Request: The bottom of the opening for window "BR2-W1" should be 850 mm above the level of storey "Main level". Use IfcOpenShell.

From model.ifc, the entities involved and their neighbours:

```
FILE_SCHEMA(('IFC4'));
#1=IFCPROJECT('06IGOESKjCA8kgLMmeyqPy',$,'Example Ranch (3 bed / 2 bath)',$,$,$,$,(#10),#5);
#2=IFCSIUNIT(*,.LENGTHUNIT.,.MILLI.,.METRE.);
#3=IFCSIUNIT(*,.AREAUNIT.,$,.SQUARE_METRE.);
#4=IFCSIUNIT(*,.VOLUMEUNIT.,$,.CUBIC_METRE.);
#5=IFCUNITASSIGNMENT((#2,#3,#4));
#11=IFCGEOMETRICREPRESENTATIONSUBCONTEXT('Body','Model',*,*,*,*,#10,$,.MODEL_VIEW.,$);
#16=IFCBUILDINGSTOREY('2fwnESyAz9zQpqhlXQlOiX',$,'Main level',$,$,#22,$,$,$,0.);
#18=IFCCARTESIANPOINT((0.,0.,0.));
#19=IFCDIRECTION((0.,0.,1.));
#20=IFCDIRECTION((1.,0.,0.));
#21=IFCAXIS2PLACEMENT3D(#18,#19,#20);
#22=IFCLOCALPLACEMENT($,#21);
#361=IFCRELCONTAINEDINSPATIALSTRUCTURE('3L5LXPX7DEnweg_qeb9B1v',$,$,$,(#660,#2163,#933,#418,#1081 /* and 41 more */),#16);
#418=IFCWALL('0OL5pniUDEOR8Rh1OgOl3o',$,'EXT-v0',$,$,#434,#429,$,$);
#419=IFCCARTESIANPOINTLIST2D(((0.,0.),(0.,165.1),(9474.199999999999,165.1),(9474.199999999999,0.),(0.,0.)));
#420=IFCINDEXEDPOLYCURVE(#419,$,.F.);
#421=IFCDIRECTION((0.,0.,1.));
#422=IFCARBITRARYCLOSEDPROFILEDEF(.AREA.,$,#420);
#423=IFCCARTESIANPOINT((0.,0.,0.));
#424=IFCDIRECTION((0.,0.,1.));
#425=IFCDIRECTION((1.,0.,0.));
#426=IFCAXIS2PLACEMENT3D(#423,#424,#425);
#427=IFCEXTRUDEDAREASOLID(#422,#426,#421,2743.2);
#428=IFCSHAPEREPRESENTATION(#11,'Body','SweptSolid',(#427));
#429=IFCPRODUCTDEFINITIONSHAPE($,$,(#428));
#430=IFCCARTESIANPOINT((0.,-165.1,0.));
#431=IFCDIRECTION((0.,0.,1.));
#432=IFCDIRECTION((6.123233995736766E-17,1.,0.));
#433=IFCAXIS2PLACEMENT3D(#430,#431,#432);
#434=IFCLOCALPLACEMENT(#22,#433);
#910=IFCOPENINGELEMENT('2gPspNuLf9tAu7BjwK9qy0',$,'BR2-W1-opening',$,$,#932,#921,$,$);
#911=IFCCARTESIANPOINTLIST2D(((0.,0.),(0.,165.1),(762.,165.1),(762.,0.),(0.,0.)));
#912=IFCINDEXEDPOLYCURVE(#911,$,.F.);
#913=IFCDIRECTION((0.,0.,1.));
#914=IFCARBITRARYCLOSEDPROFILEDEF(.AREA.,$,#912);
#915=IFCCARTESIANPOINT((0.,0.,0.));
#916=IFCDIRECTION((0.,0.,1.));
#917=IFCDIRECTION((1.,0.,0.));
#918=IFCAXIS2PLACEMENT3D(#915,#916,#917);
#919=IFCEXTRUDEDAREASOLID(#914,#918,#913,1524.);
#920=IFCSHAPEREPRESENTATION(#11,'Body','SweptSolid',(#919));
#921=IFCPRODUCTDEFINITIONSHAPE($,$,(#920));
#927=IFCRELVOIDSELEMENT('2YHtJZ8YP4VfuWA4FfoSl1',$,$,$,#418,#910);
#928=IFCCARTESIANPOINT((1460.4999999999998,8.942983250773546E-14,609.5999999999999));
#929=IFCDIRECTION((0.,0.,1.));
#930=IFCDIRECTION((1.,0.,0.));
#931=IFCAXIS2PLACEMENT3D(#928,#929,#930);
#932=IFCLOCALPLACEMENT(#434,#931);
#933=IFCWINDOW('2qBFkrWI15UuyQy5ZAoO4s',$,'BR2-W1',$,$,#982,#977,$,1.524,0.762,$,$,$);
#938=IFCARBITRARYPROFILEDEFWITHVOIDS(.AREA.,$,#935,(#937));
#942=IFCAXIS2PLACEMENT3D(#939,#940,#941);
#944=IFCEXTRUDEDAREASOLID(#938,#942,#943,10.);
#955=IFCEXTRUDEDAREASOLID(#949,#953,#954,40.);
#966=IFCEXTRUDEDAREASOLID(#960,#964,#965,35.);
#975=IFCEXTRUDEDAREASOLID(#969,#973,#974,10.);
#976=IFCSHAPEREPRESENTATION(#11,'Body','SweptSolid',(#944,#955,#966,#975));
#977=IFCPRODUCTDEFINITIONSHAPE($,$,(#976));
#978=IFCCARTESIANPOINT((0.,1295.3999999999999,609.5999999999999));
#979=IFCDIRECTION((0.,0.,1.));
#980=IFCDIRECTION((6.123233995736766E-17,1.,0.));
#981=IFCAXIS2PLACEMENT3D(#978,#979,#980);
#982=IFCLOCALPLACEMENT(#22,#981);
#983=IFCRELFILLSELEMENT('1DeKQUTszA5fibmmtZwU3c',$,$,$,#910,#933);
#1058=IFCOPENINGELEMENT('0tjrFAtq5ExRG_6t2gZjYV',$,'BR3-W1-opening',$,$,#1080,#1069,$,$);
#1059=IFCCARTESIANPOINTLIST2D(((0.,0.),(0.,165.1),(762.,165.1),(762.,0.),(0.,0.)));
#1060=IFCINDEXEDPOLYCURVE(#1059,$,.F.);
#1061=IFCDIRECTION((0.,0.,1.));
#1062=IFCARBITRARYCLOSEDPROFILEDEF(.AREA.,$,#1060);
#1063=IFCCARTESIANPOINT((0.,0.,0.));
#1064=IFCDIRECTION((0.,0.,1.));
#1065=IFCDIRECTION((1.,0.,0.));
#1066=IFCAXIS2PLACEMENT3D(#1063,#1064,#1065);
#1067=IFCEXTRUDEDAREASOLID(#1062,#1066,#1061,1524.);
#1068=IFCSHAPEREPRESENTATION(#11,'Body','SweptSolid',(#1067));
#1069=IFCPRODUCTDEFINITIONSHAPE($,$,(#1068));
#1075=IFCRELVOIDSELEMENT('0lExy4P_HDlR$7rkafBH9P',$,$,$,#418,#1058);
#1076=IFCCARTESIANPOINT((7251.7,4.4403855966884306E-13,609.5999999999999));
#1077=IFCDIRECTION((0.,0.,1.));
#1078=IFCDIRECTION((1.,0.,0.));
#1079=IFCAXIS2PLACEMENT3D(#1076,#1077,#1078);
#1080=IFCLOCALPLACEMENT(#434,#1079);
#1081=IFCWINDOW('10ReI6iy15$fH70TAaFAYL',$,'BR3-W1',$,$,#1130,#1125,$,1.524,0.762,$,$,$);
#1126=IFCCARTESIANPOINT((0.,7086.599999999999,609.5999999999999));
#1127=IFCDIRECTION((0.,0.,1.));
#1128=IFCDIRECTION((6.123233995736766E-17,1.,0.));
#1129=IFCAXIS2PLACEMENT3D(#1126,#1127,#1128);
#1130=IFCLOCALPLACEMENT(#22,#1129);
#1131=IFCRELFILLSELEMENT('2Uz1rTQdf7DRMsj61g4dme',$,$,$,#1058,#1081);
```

```python
import numpy as np
import ifcopenshell
import ifcopenshell.api.geometry
import ifcopenshell.geom
import ifcopenshell.util.element
import ifcopenshell.util.placement
import ifcopenshell.util.shape
import ifcopenshell.util.unit

model = ifcopenshell.open("model.ifc")
unit_scale = ifcopenshell.util.unit.calculate_unit_scale(model)

window = model.by_guid("2qBFkrWI15UuyQy5ZAoO4s")
opening = window.FillsVoids[0].RelatingOpeningElement
storey = ifcopenshell.util.element.get_container(window, ifc_class="IfcBuildingStorey")
level = ifcopenshell.util.placement.get_local_placement(storey.ObjectPlacement)[2, 3]

# The opening's origin need not be at the sill, so measure its lowest point.
shape = ifcopenshell.geom.create_shape(ifcopenshell.geom.settings(), opening)
bottom = ifcopenshell.util.shape.get_shape_bottom_elevation(shape, shape.geometry) / unit_scale
dz = level + 0.85 / unit_scale - bottom

shift = np.array([0.0, 0.0, dz])
# The window is not placed relative to its opening, so move both.
for product in (opening, window):
    matrix = ifcopenshell.util.placement.get_local_placement(product.ObjectPlacement)
    matrix[:3, 3] += shift
    ifcopenshell.api.geometry.edit_object_placement(model, product=product, matrix=matrix, is_si=False)

print(f"moved by {dz * unit_scale:+.3f} m")

model.write("model_edited.ifc")
```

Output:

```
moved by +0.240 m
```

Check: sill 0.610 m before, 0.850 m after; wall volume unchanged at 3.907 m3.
